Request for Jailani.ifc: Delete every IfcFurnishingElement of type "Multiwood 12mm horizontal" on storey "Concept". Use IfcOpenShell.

First a look at what the model holds.

```python
import ifcopenshell
import ifcopenshell.util.element

model = ifcopenshell.open("Jailani.ifc")
print(model.schema)
storey = next(s for s in model.by_type("IfcBuildingStorey") if s.Name == "Concept")
furniture = [e for e in ifcopenshell.util.element.get_decomposition(storey) if e.is_a("IfcFurnishingElement")]
seen = {}
for e in furniture:
    element_type = ifcopenshell.util.element.get_type(e)
    name = element_type.Name if element_type not in (None, e) else None
    seen[name] = seen.get(name, 0) + 1
for name, count in sorted(seen.items(), key=str):
    print(count, "x", name)
```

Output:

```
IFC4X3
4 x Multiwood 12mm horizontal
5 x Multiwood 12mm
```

```python
import ifcopenshell
import ifcopenshell.api.root
import ifcopenshell.util.element

model = ifcopenshell.open("Jailani.ifc")

storey = next(s for s in model.by_type("IfcBuildingStorey") if s.Name == "Concept")
furniture = [e for e in ifcopenshell.util.element.get_decomposition(storey) if e.is_a("IfcFurnishingElement")]
targets = [e for e in furniture if (t := ifcopenshell.util.element.get_type(e)) not in (None, e) and t.Name == "Multiwood 12mm horizontal"]

for e in targets:
    ifcopenshell.api.root.remove_product(model, product=e)
print(len(targets), "removed")

model.write("Jailani-out.ifc")
```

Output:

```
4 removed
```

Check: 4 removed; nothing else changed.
